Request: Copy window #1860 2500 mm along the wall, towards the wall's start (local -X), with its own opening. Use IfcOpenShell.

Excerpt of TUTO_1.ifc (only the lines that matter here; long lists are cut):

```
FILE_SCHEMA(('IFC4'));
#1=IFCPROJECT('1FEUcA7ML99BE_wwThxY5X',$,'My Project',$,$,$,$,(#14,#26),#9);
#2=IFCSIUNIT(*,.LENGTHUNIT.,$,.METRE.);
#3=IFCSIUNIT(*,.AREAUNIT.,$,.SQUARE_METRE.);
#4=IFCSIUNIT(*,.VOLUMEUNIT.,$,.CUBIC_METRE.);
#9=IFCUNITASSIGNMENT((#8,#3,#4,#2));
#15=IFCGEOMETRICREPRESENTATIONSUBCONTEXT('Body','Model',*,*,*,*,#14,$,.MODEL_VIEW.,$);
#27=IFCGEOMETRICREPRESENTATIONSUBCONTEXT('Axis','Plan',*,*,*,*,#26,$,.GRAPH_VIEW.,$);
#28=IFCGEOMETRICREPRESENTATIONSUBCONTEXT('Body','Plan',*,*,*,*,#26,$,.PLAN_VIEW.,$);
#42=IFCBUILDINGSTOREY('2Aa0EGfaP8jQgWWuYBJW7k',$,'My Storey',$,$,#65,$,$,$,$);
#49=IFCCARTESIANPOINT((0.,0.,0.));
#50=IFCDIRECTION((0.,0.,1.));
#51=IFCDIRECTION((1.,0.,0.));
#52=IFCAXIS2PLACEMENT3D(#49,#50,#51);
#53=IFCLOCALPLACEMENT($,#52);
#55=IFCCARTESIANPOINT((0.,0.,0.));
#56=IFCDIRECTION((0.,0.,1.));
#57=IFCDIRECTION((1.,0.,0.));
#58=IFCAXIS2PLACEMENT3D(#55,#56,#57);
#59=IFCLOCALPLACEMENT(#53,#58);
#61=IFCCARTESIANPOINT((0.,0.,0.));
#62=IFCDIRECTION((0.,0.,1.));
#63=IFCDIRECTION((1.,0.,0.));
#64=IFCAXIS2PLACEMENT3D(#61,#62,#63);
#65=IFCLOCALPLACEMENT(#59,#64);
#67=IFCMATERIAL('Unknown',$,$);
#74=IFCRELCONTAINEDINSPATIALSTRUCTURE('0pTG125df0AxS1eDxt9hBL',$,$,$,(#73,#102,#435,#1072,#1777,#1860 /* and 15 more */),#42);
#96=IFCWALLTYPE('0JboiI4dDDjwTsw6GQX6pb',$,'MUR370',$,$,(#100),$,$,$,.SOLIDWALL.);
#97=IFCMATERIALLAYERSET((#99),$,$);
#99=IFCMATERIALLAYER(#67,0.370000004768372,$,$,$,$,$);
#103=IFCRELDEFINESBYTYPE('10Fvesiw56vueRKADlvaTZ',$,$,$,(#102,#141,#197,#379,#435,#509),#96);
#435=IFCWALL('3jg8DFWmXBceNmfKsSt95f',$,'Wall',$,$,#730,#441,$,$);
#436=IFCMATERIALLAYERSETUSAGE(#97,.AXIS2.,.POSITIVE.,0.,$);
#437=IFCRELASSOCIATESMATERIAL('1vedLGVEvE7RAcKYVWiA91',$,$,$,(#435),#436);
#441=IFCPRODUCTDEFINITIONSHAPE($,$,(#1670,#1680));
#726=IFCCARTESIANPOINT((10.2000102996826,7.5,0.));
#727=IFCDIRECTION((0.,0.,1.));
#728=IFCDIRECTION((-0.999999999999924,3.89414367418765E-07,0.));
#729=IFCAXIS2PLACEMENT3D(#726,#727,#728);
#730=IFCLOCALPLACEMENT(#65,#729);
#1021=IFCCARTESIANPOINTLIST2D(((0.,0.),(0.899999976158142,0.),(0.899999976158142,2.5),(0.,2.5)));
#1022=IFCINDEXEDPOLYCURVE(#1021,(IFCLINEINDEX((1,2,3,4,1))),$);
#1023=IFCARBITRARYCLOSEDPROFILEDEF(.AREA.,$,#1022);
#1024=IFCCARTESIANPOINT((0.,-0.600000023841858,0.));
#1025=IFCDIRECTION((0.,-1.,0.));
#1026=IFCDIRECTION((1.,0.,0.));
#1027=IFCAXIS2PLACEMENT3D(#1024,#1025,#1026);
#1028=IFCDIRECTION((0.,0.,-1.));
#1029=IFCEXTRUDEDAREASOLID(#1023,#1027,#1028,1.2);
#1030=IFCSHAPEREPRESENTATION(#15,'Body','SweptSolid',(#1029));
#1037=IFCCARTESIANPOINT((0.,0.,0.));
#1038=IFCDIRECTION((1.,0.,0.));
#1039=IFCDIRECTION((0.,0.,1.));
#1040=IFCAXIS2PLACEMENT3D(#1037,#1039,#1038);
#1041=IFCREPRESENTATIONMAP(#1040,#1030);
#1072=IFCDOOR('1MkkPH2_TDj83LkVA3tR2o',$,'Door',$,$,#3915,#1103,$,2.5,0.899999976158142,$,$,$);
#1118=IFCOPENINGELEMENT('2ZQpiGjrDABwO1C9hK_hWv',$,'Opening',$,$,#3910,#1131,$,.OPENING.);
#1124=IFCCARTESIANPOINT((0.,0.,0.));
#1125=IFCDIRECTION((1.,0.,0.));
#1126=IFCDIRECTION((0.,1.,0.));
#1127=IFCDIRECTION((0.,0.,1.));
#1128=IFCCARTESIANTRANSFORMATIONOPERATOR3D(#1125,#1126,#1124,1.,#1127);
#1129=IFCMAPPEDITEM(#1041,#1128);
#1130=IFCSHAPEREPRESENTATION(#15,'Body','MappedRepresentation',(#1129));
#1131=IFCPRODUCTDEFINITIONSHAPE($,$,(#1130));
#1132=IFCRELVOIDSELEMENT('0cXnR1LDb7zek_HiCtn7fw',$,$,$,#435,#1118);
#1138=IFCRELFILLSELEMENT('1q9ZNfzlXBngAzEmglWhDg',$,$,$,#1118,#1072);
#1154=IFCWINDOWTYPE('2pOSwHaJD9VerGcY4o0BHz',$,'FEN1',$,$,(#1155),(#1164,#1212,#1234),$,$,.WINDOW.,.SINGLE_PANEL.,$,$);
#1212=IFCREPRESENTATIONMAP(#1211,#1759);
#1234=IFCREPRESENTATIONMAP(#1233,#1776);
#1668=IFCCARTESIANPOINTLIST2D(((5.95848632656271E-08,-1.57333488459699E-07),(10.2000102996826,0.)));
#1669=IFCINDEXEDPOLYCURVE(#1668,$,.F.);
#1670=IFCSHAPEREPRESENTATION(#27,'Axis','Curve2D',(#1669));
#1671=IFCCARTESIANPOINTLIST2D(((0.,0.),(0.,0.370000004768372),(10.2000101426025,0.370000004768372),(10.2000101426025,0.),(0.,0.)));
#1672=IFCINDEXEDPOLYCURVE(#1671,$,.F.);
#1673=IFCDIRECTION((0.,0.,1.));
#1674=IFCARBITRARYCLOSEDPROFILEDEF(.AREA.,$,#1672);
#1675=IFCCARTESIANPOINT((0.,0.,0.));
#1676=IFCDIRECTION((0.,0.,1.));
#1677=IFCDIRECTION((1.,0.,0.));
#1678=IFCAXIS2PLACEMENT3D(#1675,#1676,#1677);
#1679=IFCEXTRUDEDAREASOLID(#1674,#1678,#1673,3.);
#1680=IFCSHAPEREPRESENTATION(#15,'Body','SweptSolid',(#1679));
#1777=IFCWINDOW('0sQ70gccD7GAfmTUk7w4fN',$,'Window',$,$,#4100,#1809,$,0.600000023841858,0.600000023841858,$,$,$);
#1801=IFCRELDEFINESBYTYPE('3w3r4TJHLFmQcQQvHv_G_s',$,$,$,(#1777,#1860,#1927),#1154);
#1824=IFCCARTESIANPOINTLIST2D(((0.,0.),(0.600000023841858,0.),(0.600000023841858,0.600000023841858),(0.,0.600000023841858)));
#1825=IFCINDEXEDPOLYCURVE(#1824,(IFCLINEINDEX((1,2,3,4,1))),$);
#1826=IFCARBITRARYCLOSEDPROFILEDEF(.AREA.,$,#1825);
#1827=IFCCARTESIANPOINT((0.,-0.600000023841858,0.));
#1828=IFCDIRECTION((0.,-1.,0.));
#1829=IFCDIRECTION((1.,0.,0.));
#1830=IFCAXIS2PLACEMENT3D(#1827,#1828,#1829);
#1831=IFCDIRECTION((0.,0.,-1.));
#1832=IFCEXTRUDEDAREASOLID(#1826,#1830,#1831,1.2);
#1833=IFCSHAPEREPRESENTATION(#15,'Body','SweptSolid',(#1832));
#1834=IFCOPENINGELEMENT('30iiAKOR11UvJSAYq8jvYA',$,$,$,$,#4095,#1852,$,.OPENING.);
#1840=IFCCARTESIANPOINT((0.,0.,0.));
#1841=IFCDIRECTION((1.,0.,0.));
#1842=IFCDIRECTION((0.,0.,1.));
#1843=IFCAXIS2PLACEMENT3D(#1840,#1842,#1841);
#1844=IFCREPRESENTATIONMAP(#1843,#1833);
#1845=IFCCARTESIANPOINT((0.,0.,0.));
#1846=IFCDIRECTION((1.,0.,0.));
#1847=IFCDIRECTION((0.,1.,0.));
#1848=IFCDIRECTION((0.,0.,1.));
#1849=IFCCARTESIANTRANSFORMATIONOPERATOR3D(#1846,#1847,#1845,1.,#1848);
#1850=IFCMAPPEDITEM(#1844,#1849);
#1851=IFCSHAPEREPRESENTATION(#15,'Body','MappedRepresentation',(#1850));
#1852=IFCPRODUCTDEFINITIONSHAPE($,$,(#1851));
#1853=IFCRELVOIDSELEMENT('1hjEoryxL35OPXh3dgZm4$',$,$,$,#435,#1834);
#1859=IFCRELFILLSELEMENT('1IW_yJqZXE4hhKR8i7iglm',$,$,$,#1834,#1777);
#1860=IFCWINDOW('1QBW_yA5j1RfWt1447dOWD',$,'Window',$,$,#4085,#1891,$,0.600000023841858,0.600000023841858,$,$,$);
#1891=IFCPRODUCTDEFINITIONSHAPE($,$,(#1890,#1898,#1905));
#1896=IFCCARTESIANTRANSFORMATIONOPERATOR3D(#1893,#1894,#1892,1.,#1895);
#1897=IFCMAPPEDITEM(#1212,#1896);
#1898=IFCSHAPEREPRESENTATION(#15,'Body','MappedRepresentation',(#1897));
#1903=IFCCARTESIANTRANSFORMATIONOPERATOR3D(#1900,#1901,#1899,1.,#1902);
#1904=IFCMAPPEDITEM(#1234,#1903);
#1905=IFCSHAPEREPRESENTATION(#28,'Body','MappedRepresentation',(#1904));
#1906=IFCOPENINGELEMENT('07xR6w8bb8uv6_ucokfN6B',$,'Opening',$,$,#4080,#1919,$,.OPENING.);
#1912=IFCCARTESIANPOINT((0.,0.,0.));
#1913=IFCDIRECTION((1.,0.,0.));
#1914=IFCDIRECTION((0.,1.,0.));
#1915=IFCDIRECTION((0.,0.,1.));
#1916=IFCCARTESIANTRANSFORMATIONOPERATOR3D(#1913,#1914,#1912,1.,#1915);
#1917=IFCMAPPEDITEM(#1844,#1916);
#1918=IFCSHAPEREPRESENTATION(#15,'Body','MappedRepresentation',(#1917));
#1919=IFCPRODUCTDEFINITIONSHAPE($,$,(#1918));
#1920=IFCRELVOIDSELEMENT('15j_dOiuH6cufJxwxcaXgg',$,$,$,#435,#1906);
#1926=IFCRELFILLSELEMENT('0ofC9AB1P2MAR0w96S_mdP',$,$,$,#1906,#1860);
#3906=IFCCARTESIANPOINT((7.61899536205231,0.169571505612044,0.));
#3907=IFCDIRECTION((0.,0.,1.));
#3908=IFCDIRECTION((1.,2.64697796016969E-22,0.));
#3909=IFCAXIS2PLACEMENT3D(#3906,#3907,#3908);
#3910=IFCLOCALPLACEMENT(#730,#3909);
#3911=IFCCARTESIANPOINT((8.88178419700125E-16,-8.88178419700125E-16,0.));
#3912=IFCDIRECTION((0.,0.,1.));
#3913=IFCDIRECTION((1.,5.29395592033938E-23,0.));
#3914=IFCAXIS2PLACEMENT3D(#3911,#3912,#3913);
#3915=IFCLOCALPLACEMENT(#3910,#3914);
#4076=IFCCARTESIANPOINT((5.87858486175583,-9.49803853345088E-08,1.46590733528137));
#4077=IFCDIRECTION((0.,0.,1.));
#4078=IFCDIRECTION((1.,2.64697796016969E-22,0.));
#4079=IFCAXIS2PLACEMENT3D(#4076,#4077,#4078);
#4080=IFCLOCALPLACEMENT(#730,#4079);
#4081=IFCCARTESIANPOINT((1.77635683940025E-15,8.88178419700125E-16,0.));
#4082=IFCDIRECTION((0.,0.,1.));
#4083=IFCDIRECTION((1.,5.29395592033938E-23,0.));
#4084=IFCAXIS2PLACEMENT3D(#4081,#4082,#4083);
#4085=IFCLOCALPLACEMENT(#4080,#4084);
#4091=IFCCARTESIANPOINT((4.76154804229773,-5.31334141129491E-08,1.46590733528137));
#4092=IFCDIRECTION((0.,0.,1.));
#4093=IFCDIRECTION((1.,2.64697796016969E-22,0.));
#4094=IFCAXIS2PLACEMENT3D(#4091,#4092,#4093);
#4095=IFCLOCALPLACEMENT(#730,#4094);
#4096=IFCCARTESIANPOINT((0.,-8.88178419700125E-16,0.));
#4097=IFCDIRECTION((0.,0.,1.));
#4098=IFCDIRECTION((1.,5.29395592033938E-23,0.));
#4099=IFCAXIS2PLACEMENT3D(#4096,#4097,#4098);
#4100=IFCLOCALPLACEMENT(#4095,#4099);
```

```python
import ifcopenshell
import ifcopenshell.api.feature
import ifcopenshell.api.geometry
import ifcopenshell.api.root
import ifcopenshell.geom
import ifcopenshell.util.element
import ifcopenshell.util.placement
import ifcopenshell.util.shape

model = ifcopenshell.open("TUTO_1.ifc")
settings = ifcopenshell.geom.settings()


def volume(element):
    """Net volume in cubic metres, openings subtracted."""
    shape = ifcopenshell.geom.create_shape(settings, element)
    return ifcopenshell.util.shape.get_volume(shape.geometry)


window = model.by_id(1860)
opening = window.FillsVoids[0].RelatingOpeningElement
wall = opening.VoidsElements[0].RelatingBuildingElement
before = volume(wall)
shift = ifcopenshell.util.placement.get_local_placement(wall.ObjectPlacement)[:3, 0] * -2.5

# copy_class copies the void relationship, type, container and properties, but no geometry.
new_opening = ifcopenshell.api.root.copy_class(model, product=opening)
new_opening.Representation = ifcopenshell.util.element.copy_deep(
    model, opening.Representation, exclude=["IfcGeometricRepresentationContext", "IfcRepresentationMap"]
)
new_window = ifcopenshell.api.root.copy_class(model, product=window)
new_window.Representation = ifcopenshell.util.element.copy_deep(
    model, window.Representation, exclude=["IfcGeometricRepresentationContext", "IfcRepresentationMap"]
)
ifcopenshell.api.feature.add_filling(model, opening=new_opening, element=new_window)

for old, new in ((opening, new_opening), (window, new_window)):
    matrix = ifcopenshell.util.placement.get_local_placement(old.ObjectPlacement)
    matrix[:3, 3] += shift
    ifcopenshell.api.geometry.edit_object_placement(model, product=new, matrix=matrix, is_si=False)

after = volume(wall)

print(f"wall volume {before:.3f} -> {after:.3f} m3")

model.write("TUTO_1_v2.ifc")
```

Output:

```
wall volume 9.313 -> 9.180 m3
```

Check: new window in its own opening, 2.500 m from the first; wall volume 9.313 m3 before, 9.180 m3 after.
